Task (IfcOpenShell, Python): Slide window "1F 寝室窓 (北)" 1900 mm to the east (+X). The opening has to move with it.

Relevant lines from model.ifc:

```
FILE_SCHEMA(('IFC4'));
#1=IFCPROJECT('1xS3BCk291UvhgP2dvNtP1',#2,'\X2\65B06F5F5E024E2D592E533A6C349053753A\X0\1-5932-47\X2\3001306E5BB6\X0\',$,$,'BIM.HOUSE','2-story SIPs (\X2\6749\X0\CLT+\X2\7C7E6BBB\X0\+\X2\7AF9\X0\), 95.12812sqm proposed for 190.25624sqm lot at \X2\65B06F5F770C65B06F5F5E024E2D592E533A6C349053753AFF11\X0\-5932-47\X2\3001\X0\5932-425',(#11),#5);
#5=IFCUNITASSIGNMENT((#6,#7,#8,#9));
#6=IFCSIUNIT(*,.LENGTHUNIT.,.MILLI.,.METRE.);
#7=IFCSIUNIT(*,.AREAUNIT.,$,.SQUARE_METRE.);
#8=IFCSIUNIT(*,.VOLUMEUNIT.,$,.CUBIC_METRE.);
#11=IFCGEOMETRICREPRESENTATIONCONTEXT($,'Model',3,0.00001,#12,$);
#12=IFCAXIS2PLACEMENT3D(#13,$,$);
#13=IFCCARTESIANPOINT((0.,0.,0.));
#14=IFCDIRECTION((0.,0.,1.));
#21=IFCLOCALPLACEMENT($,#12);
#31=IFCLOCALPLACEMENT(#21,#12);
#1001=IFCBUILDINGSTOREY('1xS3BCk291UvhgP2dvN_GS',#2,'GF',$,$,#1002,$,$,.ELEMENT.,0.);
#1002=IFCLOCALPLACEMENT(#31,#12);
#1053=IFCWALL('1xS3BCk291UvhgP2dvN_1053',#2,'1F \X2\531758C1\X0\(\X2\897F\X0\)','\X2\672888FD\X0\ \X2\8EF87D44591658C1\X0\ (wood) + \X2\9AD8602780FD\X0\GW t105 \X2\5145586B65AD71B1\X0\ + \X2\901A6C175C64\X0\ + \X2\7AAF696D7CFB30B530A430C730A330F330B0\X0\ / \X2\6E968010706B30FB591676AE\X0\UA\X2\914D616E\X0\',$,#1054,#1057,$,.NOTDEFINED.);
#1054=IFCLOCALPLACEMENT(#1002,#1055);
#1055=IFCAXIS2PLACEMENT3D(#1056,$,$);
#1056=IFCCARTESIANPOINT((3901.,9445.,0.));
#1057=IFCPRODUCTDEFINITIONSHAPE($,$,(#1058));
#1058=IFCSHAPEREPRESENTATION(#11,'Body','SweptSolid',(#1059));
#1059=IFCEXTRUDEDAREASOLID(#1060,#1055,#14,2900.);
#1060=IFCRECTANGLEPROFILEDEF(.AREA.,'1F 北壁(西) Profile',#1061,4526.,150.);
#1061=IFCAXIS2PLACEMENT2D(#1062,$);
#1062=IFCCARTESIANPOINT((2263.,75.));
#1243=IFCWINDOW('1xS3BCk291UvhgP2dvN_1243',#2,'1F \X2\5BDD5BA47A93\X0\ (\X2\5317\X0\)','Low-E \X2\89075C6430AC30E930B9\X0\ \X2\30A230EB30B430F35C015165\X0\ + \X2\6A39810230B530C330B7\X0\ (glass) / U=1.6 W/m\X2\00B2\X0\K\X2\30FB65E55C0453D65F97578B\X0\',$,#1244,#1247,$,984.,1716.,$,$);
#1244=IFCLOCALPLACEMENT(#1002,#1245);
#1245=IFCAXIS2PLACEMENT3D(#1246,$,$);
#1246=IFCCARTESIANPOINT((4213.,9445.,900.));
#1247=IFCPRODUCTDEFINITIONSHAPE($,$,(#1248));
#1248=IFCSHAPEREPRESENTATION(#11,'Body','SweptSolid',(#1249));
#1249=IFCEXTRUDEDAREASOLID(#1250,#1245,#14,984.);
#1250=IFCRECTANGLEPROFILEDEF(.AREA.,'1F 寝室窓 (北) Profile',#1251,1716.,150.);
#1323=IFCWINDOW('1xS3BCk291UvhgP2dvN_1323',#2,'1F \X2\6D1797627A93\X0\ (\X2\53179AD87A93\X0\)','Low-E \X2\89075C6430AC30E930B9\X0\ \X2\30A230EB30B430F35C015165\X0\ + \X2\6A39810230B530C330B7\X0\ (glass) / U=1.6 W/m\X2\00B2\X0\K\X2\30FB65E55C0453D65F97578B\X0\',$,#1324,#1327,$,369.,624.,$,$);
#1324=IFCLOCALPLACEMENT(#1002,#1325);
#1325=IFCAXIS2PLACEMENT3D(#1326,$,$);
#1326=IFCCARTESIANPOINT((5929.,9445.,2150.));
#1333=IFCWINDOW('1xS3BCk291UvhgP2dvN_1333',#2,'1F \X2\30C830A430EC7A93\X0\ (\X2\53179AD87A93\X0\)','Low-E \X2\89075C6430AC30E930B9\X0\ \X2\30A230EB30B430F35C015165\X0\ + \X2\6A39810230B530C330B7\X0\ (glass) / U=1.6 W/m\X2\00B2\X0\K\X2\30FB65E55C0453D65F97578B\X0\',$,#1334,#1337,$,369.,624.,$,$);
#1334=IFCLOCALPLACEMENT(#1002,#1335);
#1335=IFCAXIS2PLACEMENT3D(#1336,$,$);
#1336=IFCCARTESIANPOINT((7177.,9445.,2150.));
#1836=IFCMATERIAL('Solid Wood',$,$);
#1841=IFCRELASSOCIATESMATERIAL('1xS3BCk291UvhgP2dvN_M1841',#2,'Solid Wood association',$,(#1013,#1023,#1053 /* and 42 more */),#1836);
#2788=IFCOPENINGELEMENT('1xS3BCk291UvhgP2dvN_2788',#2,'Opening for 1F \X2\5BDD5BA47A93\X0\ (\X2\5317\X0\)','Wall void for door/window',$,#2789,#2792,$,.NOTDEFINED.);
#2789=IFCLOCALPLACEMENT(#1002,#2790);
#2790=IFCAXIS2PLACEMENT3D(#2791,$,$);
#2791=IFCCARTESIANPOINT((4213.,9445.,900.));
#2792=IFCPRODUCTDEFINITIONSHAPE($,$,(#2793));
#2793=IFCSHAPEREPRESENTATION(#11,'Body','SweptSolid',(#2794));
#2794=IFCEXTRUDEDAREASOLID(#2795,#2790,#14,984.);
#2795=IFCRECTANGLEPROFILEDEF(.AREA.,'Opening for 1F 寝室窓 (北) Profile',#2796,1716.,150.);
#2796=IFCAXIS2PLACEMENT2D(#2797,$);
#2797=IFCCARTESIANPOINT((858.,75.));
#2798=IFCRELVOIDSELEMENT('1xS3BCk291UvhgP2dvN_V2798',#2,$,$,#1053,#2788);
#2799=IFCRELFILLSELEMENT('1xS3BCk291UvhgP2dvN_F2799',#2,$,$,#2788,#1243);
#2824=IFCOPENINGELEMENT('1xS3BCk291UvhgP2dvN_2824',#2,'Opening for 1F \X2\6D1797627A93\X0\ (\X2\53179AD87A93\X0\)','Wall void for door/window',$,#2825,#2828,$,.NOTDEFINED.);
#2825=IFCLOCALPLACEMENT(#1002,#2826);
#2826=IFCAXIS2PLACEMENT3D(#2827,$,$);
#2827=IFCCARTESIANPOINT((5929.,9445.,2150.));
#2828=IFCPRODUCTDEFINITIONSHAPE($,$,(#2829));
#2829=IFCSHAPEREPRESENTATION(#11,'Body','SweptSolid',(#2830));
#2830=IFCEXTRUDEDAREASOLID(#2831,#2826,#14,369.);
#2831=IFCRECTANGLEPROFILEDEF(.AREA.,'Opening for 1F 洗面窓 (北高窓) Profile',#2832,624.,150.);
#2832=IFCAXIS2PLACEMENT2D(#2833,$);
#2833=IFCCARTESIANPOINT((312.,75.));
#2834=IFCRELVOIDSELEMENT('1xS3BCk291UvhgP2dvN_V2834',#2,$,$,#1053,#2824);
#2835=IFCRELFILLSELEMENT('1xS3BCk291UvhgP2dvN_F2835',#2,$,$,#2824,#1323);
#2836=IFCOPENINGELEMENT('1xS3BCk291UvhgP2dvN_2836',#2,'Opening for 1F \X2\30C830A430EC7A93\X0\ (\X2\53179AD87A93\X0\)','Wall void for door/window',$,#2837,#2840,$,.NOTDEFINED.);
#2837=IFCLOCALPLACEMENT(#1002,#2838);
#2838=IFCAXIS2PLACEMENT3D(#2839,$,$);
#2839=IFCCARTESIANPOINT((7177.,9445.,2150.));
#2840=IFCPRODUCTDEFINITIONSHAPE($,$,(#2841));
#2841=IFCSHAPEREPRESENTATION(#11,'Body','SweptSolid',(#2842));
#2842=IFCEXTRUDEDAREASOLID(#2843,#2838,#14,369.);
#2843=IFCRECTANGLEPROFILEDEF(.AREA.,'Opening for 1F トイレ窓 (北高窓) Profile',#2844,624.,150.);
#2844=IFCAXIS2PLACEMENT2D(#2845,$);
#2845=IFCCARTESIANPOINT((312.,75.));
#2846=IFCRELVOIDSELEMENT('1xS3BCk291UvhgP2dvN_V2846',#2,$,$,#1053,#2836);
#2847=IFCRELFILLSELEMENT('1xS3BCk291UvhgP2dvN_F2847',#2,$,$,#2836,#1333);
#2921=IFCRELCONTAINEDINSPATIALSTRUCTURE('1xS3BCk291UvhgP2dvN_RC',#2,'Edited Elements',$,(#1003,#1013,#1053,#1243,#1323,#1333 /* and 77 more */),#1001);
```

```python
import ifcopenshell
import ifcopenshell.api.geometry
import ifcopenshell.util.placement

model = ifcopenshell.open("model.ifc")

window = model.by_guid("1xS3BCk291UvhgP2dvN_1243")
opening = window.FillsVoids[0].RelatingOpeningElement
wall = opening.VoidsElements[0].RelatingBuildingElement

wall_matrix = ifcopenshell.util.placement.get_local_placement(wall.ObjectPlacement)
shift = wall_matrix[:3, 0] * 1900.0
before = ifcopenshell.util.placement.get_local_placement(window.ObjectPlacement)[:3, 3].copy()

# The window is not placed relative to its opening, so move both.
for product in (opening, window):
    matrix = ifcopenshell.util.placement.get_local_placement(product.ObjectPlacement)
    matrix[:3, 3] += shift
    ifcopenshell.api.geometry.edit_object_placement(model, product=product, matrix=matrix, is_si=False)

after = ifcopenshell.util.placement.get_local_placement(window.ObjectPlacement)[:3, 3]
print("window moved by", (after - before).round(3) + 0.0)

model.write("model_edited.ifc")
```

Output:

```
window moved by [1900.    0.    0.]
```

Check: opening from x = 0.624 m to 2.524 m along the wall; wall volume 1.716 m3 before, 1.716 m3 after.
